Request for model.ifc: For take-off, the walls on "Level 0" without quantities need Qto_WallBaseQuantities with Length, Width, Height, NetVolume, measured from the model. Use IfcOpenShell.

First a look at what the model holds.

```python
import ifcopenshell
import ifcopenshell.util.element
import ifcopenshell.util.unit

model = ifcopenshell.open("model.ifc")
print(model.schema)
for unit_type in ("LENGTHUNIT", "AREAUNIT", "VOLUMEUNIT"):
    print(unit_type, ifcopenshell.util.unit.calculate_unit_scale(model, unit_type))
storey = next(s for s in model.by_type("IfcBuildingStorey") if s.Name == "Level 0")
walls = [e for e in ifcopenshell.util.element.get_decomposition(storey) if e.is_a("IfcWall")]
for e in sorted(walls, key=lambda e: e.id()):
    print(e.id(), e.is_a(), e.Name, list(ifcopenshell.util.element.get_psets(e, qtos_only=True)), sep=" | ")
```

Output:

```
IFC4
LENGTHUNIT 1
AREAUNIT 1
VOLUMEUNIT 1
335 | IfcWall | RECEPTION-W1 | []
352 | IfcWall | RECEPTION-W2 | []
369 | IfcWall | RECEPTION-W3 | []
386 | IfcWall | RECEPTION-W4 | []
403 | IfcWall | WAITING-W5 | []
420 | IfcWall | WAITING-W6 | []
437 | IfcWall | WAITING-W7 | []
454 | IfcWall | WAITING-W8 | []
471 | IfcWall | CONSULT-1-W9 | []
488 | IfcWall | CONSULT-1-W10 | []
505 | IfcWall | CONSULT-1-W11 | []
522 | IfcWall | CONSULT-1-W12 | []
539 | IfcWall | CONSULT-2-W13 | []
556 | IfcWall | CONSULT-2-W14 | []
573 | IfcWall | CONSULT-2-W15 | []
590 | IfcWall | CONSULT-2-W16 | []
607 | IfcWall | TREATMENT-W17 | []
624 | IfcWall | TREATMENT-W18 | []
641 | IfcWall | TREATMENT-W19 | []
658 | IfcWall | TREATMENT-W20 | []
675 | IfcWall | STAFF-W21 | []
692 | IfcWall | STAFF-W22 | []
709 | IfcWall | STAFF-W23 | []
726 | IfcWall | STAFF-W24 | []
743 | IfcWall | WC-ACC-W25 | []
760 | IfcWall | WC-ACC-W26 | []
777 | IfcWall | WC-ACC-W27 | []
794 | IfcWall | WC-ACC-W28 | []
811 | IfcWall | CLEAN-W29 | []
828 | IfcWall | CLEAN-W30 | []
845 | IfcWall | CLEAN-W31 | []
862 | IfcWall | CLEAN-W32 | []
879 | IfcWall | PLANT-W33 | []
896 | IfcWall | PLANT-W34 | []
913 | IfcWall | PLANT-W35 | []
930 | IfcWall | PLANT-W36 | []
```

```python
import ifcopenshell
import ifcopenshell.api.pset
import ifcopenshell.geom
import ifcopenshell.util.element
import ifcopenshell.util.shape
import ifcopenshell.util.unit

model = ifcopenshell.open("model.ifc")
unit_scale = ifcopenshell.util.unit.calculate_unit_scale(model)
volume_scale = ifcopenshell.util.unit.calculate_unit_scale(model, "VOLUMEUNIT")
settings = ifcopenshell.geom.settings()

storey = next(s for s in model.by_type("IfcBuildingStorey") if s.Name == "Level 0")
walls = [e for e in ifcopenshell.util.element.get_decomposition(storey) if e.is_a("IfcWall")]

for e in sorted(walls, key=lambda e: e.id()):
    if ifcopenshell.util.element.get_psets(e, qtos_only=True, should_inherit=False):
        continue
    # Geometry comes back in metres, in the element's own axes.
    shape = ifcopenshell.geom.create_shape(settings, e)
    values = {
        "Length": ifcopenshell.util.shape.get_x(shape.geometry) / unit_scale,
        "Width": ifcopenshell.util.shape.get_y(shape.geometry) / unit_scale,
        "Height": ifcopenshell.util.shape.get_z(shape.geometry) / unit_scale,
        "NetVolume": ifcopenshell.util.shape.get_volume(shape.geometry) / volume_scale,
    }
    qto = ifcopenshell.api.pset.add_qto(model, product=e, name="Qto_WallBaseQuantities")
    ifcopenshell.api.pset.edit_qto(model, qto=qto, properties=values)
    print(e.id(), {k: round(v, 3) for k, v in values.items()})

model.write("model_updated.ifc")
```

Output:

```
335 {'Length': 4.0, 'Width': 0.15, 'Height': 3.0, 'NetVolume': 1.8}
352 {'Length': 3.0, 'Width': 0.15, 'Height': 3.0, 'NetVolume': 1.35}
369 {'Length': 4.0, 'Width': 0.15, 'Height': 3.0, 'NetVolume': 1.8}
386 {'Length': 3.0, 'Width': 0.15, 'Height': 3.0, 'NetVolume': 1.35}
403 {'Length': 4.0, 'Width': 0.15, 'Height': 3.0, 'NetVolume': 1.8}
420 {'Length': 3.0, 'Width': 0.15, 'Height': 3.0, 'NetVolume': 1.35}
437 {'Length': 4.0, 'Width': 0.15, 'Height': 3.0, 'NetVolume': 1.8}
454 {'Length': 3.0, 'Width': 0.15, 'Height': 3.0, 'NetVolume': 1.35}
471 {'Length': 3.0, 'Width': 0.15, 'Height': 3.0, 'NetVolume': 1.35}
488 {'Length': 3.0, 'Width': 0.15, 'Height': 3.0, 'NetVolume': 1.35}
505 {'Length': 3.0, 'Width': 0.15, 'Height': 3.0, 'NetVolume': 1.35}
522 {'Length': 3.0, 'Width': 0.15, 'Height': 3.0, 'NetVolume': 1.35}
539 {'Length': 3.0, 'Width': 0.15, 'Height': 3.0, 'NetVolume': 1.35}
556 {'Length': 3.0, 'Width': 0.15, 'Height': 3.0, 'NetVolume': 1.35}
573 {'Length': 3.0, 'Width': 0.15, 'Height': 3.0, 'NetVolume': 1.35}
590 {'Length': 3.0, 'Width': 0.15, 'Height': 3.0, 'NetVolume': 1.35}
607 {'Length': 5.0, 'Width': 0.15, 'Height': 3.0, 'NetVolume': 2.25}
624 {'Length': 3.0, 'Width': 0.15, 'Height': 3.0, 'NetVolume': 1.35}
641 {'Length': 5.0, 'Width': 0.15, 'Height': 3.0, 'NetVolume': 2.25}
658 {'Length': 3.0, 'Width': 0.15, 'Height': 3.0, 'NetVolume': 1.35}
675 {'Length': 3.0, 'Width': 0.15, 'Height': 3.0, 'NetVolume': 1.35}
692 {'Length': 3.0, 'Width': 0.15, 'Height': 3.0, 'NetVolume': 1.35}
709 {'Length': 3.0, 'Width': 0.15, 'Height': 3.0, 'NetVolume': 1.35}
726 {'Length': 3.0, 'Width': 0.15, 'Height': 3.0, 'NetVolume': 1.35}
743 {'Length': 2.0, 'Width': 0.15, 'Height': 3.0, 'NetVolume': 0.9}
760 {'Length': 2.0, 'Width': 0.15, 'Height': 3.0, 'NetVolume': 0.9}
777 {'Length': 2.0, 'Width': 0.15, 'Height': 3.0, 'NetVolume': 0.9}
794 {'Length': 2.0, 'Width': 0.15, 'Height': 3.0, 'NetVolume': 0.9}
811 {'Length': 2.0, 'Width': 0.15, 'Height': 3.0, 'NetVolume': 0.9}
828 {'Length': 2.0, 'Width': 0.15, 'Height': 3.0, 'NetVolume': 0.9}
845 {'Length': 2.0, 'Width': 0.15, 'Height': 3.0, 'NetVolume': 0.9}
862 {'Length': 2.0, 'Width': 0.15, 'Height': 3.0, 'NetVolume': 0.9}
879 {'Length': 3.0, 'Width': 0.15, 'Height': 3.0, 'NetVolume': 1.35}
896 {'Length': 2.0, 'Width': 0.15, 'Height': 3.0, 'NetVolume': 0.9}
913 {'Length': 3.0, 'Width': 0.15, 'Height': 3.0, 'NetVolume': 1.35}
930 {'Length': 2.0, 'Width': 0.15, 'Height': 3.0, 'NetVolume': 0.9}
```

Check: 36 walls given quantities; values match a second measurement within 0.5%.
